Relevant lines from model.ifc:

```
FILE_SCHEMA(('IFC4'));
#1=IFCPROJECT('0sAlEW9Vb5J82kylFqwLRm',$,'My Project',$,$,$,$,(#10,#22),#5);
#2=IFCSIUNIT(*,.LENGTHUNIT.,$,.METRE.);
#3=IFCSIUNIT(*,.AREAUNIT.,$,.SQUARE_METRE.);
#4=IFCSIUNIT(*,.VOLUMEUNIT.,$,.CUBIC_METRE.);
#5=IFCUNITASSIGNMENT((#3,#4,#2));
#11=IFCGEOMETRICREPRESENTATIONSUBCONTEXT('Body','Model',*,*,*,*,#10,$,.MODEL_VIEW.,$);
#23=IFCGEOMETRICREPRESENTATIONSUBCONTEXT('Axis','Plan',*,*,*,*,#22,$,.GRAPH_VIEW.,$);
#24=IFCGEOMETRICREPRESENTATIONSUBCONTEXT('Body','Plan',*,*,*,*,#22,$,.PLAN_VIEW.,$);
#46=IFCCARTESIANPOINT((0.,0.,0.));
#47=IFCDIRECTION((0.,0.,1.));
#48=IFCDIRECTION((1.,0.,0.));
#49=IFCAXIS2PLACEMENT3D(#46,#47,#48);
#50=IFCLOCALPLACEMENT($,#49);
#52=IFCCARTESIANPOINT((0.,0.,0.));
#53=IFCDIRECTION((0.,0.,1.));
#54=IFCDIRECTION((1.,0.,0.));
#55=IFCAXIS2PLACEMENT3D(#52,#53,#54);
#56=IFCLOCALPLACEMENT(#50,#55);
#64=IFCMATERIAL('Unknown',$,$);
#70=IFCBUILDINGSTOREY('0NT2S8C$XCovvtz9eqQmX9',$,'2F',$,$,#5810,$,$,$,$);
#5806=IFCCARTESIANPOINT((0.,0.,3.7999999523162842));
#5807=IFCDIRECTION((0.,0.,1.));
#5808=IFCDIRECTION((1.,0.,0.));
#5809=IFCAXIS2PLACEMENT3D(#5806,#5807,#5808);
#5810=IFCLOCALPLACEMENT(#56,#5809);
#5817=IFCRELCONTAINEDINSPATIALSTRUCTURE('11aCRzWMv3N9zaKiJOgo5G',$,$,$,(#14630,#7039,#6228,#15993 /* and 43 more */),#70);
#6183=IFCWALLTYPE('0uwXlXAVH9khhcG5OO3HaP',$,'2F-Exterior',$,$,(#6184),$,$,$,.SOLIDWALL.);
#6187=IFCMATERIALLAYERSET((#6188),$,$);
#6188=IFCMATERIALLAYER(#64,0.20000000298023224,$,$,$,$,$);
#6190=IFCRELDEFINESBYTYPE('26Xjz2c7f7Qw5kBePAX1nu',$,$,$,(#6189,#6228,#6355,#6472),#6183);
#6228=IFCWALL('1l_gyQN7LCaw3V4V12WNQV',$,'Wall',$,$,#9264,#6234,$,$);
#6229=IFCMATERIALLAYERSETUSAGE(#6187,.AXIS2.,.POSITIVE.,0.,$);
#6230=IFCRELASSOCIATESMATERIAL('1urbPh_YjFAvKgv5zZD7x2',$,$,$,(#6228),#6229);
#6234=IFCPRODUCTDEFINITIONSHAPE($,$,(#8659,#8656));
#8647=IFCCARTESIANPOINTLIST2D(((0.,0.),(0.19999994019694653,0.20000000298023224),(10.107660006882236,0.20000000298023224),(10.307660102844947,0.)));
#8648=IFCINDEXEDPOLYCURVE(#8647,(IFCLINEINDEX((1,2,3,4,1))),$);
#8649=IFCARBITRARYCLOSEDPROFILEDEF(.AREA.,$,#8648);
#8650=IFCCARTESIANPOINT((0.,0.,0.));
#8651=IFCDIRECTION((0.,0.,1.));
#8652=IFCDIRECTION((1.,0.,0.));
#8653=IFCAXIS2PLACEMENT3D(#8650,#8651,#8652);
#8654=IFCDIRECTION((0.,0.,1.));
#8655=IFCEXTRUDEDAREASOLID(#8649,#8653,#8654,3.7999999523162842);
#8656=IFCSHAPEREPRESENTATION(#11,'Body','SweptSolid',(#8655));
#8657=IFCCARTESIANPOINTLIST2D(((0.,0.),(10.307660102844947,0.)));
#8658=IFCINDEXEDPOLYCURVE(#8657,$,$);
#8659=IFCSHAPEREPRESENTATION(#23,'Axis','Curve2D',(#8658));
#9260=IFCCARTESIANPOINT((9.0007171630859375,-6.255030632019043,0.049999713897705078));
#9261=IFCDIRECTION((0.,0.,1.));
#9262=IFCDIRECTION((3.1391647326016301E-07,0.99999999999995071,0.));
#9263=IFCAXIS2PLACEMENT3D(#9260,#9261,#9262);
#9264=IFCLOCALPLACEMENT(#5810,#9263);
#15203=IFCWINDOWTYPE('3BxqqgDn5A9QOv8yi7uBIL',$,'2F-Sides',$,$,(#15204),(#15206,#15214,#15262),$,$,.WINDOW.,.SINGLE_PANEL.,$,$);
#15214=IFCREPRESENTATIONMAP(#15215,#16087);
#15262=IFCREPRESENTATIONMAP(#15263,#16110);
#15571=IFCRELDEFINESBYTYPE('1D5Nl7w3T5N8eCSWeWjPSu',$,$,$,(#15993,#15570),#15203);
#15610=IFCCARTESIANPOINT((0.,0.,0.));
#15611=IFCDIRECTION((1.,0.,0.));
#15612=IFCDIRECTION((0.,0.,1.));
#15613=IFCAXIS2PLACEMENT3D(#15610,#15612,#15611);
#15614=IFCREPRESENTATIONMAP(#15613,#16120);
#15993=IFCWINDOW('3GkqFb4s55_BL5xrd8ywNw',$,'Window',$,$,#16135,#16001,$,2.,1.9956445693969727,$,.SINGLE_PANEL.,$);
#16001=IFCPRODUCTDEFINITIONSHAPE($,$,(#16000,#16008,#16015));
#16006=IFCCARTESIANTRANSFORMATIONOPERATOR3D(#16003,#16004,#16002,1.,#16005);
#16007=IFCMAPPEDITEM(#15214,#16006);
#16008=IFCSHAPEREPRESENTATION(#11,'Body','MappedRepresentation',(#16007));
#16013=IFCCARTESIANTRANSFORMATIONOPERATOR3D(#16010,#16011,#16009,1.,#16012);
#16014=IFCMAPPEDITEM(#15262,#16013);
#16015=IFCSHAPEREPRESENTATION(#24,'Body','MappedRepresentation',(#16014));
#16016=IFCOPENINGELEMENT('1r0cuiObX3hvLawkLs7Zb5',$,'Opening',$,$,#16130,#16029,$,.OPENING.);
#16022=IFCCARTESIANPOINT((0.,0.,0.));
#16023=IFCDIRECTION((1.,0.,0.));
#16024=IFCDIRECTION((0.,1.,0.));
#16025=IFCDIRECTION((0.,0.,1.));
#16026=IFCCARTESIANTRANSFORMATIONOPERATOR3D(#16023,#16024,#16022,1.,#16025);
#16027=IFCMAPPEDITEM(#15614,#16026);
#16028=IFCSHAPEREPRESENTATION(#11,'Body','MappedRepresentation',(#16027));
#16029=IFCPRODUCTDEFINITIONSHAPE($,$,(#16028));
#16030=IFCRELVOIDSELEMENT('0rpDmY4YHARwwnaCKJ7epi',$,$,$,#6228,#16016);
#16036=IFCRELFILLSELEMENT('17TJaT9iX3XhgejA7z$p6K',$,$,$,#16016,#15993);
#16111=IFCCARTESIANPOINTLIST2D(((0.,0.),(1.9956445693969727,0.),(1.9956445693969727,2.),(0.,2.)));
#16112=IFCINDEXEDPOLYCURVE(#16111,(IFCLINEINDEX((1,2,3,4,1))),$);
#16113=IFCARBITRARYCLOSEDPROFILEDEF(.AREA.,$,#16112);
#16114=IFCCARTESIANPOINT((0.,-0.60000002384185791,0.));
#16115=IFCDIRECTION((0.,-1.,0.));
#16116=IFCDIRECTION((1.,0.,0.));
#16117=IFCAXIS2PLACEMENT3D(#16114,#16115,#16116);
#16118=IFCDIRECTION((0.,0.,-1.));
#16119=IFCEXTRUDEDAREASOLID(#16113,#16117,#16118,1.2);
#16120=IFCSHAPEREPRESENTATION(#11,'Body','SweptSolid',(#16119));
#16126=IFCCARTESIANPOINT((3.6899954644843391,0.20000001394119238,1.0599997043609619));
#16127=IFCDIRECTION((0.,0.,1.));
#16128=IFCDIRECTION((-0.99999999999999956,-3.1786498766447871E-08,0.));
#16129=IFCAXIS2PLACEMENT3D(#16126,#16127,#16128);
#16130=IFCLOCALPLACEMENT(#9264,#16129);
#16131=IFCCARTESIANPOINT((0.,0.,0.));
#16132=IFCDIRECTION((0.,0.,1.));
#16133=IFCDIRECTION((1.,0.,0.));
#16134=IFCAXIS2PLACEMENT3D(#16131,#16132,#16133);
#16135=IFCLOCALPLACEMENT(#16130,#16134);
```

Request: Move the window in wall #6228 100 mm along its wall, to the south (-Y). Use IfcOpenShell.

```python
import ifcopenshell
import ifcopenshell.api.geometry
import ifcopenshell.util.placement

model = ifcopenshell.open("model.ifc")

window = model.by_id(15993)
opening = window.FillsVoids[0].RelatingOpeningElement
wall = opening.VoidsElements[0].RelatingBuildingElement

wall_matrix = ifcopenshell.util.placement.get_local_placement(wall.ObjectPlacement)
shift = wall_matrix[:3, 0] * -0.1
before = ifcopenshell.util.placement.get_local_placement(window.ObjectPlacement)[:3, 3].copy()

# The window is placed relative to its opening, so it follows when the opening moves.
matrix = ifcopenshell.util.placement.get_local_placement(opening.ObjectPlacement)
matrix[:3, 3] += shift
ifcopenshell.api.geometry.edit_object_placement(
    model, product=opening, matrix=matrix, is_si=False, should_transform_children=True
)

after = ifcopenshell.util.placement.get_local_placement(window.ObjectPlacement)[:3, 3]
print("window moved by", (after - before).round(3) + 0.0)

model.write("model-out.ifc")
```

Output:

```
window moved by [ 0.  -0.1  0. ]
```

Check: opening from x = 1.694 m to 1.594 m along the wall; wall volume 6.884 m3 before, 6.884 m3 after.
